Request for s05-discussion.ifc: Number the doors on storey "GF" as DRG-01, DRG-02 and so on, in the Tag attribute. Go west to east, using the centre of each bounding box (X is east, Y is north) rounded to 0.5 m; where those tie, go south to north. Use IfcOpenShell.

First a look at what the model holds.

```python
import ifcopenshell
import ifcopenshell.util.element
import ifcopenshell.util.placement

model = ifcopenshell.open("s05-discussion.ifc")
print(model.schema)
storey = next(s for s in model.by_type("IfcBuildingStorey") if s.Name == "GF")
doors = [e for e in ifcopenshell.util.element.get_decomposition(storey) if e.is_a("IfcDoor")]
for e in sorted(doors, key=lambda e: e.id()):
    origin = ifcopenshell.util.placement.get_local_placement(e.ObjectPlacement)[:3, 3]
    print(e.id(), e.Tag, e.Name, origin.round(2) + 0.0, sep=" | ")
```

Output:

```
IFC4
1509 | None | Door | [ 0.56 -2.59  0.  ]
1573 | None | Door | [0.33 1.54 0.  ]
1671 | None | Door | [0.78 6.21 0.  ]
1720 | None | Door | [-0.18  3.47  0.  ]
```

```python
import ifcopenshell
import ifcopenshell.geom
import ifcopenshell.util.element
import ifcopenshell.util.shape

model = ifcopenshell.open("s05-discussion.ifc")
settings = ifcopenshell.geom.settings()
settings.set("use-world-coords", True)


def centre(element):
    shape = ifcopenshell.geom.create_shape(settings, element)
    return ifcopenshell.util.shape.get_bbox_centroid(shape.geometry)


storey = next(s for s in model.by_type("IfcBuildingStorey") if s.Name == "GF")
doors = [e for e in ifcopenshell.util.element.get_decomposition(storey) if e.is_a("IfcDoor")]

# Insertion points can sit at a corner or the storey origin, so sort by the geometry (in metres).
centres = {e: centre(e) for e in doors}
doors.sort(key=lambda e: (round(centres[e][0] / 0.5), centres[e][1]))

for i, e in enumerate(doors, start=1):
    number = f"DRG-{i:02d}"
    e.Tag = number
    print(e.id(), number)

model.write("s05-discussion_v2.ifc")
```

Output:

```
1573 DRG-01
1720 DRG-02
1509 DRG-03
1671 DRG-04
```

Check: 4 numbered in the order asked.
